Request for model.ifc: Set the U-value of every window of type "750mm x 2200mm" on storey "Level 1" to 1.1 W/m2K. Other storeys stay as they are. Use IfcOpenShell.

First a look at what the model holds.

```python
import ifcopenshell
import ifcopenshell.util.element

model = ifcopenshell.open("model.ifc")
print(model.schema)
storey = next(s for s in model.by_type("IfcBuildingStorey") if s.Name == "Level 1")
windows = [e for e in ifcopenshell.util.element.get_decomposition(storey) if e.is_a("IfcWindow")]
seen = {}
for e in windows:
    element_type = ifcopenshell.util.element.get_type(e)
    key = (element_type.Name if element_type != e and element_type else None, ifcopenshell.util.element.get_pset(e, "Pset_WindowCommon", "ThermalTransmittance"))
    seen[key] = seen.get(key, 0) + 1
for (name, value), count in sorted(seen.items(), key=str):
    print(count, "x", name, "|", value)
```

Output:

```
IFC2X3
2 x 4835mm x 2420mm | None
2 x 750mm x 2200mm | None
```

```python
import ifcopenshell
import ifcopenshell.api.pset
import ifcopenshell.util.element

model = ifcopenshell.open("model.ifc")

storey = next(s for s in model.by_type("IfcBuildingStorey") if s.Name == "Level 1")
windows = [e for e in ifcopenshell.util.element.get_decomposition(storey) if e.is_a("IfcWindow")]

count = 0
for e in windows:
    element_type = ifcopenshell.util.element.get_type(e)
    if element_type in (None, e) or element_type.Name != "750mm x 2200mm":
        continue
    # add_pset returns the element's existing set when there is one.
    pset = ifcopenshell.api.pset.add_pset(model, product=e, name="Pset_WindowCommon")
    ifcopenshell.api.pset.edit_pset(model, pset=pset, properties={"ThermalTransmittance": 1.1})
    count += 1

print(count, "windows updated")

model.write("model_rev.ifc")
```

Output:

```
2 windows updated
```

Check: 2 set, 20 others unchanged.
